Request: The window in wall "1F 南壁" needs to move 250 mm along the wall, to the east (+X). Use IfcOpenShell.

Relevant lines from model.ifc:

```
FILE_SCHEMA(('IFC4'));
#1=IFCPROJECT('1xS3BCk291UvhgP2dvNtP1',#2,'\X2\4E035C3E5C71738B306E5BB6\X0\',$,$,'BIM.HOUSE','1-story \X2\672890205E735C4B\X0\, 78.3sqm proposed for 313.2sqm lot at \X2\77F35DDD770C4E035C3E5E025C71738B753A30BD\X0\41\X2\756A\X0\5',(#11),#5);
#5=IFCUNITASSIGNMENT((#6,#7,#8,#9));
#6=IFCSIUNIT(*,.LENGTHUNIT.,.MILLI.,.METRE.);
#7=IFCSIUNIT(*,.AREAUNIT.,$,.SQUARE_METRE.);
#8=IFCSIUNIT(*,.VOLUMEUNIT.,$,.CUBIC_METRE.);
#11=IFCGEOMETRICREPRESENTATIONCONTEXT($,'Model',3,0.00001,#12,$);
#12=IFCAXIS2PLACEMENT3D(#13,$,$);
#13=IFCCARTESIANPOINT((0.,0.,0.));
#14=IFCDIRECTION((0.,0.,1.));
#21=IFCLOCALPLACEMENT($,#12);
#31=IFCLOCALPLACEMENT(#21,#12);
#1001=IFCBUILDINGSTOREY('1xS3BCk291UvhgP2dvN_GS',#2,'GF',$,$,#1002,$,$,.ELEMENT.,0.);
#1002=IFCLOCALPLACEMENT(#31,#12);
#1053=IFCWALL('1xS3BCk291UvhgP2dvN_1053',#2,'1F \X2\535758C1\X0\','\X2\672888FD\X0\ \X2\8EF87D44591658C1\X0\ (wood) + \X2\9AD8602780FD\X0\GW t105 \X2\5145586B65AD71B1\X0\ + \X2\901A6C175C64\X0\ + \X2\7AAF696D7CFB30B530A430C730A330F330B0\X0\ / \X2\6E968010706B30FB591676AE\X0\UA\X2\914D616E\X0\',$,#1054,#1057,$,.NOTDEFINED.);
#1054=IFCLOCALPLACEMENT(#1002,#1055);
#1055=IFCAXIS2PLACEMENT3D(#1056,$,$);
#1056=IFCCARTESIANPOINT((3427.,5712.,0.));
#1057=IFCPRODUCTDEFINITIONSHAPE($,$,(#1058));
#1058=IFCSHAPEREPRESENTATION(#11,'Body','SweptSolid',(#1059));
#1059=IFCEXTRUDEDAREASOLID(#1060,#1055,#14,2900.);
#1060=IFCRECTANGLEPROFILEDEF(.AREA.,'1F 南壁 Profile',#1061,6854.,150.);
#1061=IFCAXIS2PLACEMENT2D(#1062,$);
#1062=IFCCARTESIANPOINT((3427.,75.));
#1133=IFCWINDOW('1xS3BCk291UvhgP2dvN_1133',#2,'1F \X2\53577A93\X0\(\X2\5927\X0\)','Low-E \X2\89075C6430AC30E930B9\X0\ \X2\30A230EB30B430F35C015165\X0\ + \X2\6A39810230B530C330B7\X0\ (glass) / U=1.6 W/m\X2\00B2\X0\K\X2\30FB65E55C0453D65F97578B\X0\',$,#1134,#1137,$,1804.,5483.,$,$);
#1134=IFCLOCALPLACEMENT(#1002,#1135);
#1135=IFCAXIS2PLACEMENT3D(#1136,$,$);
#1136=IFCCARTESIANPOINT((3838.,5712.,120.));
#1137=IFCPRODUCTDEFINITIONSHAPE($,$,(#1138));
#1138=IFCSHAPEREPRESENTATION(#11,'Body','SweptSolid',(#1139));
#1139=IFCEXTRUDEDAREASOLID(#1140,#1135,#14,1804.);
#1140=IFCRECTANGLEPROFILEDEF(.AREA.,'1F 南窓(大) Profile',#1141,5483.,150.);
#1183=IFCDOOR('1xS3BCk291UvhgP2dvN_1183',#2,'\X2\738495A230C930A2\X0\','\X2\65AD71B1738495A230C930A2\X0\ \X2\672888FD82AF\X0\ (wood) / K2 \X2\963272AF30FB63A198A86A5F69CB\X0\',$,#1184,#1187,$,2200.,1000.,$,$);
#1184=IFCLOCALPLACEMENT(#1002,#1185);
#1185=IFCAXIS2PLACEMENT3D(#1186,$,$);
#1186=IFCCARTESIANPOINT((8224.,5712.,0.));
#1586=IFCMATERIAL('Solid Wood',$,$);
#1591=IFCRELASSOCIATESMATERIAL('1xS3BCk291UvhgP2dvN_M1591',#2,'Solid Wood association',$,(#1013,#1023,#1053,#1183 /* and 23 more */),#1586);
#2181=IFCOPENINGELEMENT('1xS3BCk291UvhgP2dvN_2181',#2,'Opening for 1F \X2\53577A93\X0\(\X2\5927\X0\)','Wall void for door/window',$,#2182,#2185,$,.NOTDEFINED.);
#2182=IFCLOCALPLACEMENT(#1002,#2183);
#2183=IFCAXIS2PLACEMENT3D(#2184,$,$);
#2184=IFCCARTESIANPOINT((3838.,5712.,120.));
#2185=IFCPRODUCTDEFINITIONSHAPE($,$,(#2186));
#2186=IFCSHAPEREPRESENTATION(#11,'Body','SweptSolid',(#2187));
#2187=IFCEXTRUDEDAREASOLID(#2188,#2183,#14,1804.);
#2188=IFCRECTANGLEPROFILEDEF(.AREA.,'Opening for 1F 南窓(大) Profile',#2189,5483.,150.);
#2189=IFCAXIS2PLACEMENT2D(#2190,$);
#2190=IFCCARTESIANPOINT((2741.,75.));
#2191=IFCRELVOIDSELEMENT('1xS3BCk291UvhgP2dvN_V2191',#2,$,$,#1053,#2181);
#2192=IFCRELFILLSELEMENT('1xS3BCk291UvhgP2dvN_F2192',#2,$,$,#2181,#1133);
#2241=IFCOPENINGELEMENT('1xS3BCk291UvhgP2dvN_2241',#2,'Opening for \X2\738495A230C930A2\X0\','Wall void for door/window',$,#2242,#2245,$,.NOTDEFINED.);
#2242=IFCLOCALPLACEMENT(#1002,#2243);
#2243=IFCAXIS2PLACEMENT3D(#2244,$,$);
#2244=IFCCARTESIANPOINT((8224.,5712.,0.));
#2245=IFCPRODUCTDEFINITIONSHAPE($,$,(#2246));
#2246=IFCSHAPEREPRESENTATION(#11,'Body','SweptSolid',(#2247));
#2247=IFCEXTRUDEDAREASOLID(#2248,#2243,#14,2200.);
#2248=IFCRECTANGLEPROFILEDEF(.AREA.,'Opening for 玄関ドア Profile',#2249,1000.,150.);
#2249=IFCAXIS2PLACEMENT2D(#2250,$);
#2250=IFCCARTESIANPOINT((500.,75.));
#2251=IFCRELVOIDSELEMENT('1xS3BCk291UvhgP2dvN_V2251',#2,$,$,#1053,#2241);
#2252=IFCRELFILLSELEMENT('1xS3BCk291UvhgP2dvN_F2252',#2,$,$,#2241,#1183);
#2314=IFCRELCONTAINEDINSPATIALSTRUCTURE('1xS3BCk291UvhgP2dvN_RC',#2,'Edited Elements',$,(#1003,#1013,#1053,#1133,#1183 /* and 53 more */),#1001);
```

```python
import ifcopenshell
import ifcopenshell.api.geometry
import ifcopenshell.util.placement

model = ifcopenshell.open("model.ifc")

window = model.by_id(1133)
opening = window.FillsVoids[0].RelatingOpeningElement
wall = opening.VoidsElements[0].RelatingBuildingElement

wall_matrix = ifcopenshell.util.placement.get_local_placement(wall.ObjectPlacement)
shift = wall_matrix[:3, 0] * 250.0
before = ifcopenshell.util.placement.get_local_placement(window.ObjectPlacement)[:3, 3].copy()

# The window is not placed relative to its opening, so move both.
for product in (opening, window):
    matrix = ifcopenshell.util.placement.get_local_placement(product.ObjectPlacement)
    matrix[:3, 3] += shift
    ifcopenshell.api.geometry.edit_object_placement(model, product=product, matrix=matrix, is_si=False)

after = ifcopenshell.util.placement.get_local_placement(window.ObjectPlacement)[:3, 3]
print("window moved by", (after - before).round(3) + 0.0)

model.write("model-out.ifc")
```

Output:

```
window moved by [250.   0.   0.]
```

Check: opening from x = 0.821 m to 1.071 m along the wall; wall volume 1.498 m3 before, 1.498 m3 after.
